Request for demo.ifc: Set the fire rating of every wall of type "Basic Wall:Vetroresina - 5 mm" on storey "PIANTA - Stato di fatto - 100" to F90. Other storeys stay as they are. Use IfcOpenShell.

First a look at what the model holds.

```python
import ifcopenshell
import ifcopenshell.util.element

model = ifcopenshell.open("demo.ifc")
print(model.schema)
storey = next(s for s in model.by_type("IfcBuildingStorey") if s.Name == "PIANTA - Stato di fatto - 100")
walls = [e for e in ifcopenshell.util.element.get_decomposition(storey) if e.is_a("IfcWall")]
seen = {}
for e in walls:
    element_type = ifcopenshell.util.element.get_type(e)
    key = (element_type.Name if element_type != e and element_type else None, ifcopenshell.util.element.get_pset(e, "Pset_WallCommon", "FireRating"))
    seen[key] = seen.get(key, 0) + 1
for (name, value), count in sorted(seen.items(), key=str):
    print(count, "x", name, "|", value)
```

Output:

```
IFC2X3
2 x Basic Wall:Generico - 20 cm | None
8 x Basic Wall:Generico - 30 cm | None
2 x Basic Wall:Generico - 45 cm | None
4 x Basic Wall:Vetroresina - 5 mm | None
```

```python
import ifcopenshell
import ifcopenshell.api.pset
import ifcopenshell.util.element

model = ifcopenshell.open("demo.ifc")

storey = next(s for s in model.by_type("IfcBuildingStorey") if s.Name == "PIANTA - Stato di fatto - 100")
walls = [e for e in ifcopenshell.util.element.get_decomposition(storey) if e.is_a("IfcWall")]

count = 0
for e in walls:
    element_type = ifcopenshell.util.element.get_type(e)
    if element_type in (None, e) or element_type.Name != "Basic Wall:Vetroresina - 5 mm":
        continue
    # add_pset returns the element's existing set when there is one.
    pset = ifcopenshell.api.pset.add_pset(model, product=e, name="Pset_WallCommon")
    ifcopenshell.api.pset.edit_pset(model, pset=pset, properties={"FireRating": "F90"})
    count += 1

print(count, "walls updated")

model.write("demo-out.ifc")
```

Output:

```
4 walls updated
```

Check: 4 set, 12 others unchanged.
